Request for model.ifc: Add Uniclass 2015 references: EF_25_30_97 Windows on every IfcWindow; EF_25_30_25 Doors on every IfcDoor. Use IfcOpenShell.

First a look at what the model holds.

```python
import ifcopenshell

model = ifcopenshell.open("model.ifc")
print(model.schema)
print("classifications:", [c.Name for c in model.by_type("IfcClassification")])
for ifc_class in ("IfcDoor", "IfcRoof", "IfcStair", "IfcWall", "IfcWindow"):
    print(ifc_class, len(model.by_type(ifc_class)))
```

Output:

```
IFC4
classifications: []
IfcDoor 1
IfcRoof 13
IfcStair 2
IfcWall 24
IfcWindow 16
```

```python
import ifcopenshell
import ifcopenshell.api.classification

model = ifcopenshell.open("model.ifc")

system = ifcopenshell.api.classification.add_classification(model, classification="Uniclass 2015")

codes = {
    "IfcWindow": ("EF_25_30_97", "Windows"),
    "IfcDoor": ("EF_25_30_25", "Doors"),
}
for ifc_class, (code, name) in codes.items():
    products = model.by_type(ifc_class)
    ifcopenshell.api.classification.add_reference(
        model, products=products, classification=system, identification=code, name=name
    )
    print(code, len(products))

model.write("model-out.ifc")
```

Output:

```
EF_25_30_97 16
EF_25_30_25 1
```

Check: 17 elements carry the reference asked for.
